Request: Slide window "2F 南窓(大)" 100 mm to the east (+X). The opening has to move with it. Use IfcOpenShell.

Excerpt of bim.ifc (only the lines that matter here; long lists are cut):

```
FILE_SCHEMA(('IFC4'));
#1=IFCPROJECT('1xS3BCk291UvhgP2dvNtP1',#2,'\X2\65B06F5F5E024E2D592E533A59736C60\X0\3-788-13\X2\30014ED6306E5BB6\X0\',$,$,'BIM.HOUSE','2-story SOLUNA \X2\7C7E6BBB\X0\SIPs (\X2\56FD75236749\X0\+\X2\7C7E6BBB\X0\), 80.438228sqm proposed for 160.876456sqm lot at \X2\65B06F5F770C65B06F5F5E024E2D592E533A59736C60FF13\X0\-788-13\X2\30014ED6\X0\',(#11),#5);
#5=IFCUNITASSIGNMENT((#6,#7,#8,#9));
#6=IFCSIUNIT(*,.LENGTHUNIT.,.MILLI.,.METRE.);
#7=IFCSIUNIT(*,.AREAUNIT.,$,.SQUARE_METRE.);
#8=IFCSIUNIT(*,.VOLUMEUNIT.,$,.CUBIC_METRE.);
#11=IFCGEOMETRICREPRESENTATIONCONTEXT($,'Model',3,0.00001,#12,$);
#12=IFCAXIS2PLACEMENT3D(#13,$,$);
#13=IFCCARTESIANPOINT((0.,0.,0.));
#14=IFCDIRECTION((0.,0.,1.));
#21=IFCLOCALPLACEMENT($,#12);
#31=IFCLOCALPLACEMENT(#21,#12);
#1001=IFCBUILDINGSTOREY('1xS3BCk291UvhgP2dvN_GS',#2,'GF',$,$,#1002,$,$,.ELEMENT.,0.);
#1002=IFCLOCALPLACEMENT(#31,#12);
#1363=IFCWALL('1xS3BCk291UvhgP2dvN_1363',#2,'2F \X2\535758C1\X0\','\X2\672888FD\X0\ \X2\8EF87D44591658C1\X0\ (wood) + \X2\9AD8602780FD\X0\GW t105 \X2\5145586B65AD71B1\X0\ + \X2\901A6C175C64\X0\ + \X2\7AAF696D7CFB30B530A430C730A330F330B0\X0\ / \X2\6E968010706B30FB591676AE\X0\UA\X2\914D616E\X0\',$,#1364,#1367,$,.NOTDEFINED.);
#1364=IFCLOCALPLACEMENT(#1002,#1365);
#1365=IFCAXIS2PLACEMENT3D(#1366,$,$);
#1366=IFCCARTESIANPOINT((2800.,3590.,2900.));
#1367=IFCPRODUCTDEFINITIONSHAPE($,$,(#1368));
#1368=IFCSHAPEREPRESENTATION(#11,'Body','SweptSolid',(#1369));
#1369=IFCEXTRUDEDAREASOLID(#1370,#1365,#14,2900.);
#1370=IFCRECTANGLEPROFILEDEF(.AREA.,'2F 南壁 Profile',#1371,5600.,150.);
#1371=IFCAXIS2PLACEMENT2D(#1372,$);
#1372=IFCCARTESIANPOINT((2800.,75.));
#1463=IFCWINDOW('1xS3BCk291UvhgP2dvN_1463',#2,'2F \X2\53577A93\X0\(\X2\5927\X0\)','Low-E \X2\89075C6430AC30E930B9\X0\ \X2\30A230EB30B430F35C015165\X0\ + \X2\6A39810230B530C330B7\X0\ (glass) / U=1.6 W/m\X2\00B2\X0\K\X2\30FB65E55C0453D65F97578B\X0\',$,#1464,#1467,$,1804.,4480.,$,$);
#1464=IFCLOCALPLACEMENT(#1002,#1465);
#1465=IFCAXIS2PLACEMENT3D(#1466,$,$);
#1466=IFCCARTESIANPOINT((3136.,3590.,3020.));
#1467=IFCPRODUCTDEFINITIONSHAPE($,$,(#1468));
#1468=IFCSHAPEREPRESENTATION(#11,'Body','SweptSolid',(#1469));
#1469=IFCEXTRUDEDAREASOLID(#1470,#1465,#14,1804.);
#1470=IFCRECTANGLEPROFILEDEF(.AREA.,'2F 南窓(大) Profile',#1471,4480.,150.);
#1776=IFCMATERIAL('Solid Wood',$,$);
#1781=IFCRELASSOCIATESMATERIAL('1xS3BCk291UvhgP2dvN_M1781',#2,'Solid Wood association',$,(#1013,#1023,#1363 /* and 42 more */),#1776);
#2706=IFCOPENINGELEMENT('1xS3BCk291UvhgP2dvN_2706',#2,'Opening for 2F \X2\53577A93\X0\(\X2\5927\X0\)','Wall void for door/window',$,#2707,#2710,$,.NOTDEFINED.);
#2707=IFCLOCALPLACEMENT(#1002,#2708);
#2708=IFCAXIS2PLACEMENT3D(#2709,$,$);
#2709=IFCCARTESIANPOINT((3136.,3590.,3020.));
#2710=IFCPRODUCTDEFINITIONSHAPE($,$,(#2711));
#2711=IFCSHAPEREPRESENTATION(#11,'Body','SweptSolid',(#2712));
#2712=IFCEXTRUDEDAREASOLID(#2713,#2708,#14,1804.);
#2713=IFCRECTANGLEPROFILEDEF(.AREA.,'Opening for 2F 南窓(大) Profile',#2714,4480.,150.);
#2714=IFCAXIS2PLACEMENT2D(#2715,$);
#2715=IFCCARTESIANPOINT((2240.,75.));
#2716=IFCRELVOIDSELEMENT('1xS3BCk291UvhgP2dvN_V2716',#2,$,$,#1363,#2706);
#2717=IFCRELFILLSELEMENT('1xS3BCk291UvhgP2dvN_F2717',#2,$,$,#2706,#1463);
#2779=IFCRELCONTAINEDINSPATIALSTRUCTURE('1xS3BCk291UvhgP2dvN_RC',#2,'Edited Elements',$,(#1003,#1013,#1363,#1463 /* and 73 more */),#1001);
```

```python
import ifcopenshell
import ifcopenshell.api.geometry
import ifcopenshell.util.placement
import ifcopenshell.util.unit

model = ifcopenshell.open("bim.ifc")
unit_scale = ifcopenshell.util.unit.calculate_unit_scale(model)

window = model.by_id(1463)
opening = window.FillsVoids[0].RelatingOpeningElement
wall = opening.VoidsElements[0].RelatingBuildingElement

wall_matrix = ifcopenshell.util.placement.get_local_placement(wall.ObjectPlacement)
shift = wall_matrix[:3, 0] * 0.1 / unit_scale
before = ifcopenshell.util.placement.get_local_placement(window.ObjectPlacement)[:3, 3].copy()

# The window is not placed relative to its opening, so move both.
for product in (opening, window):
    matrix = ifcopenshell.util.placement.get_local_placement(product.ObjectPlacement)
    matrix[:3, 3] += shift
    ifcopenshell.api.geometry.edit_object_placement(model, product=product, matrix=matrix, is_si=False)

after = ifcopenshell.util.placement.get_local_placement(window.ObjectPlacement)[:3, 3]
print("window moved by", (after - before).round(3) + 0.0)

model.write("bim-out.ifc")
```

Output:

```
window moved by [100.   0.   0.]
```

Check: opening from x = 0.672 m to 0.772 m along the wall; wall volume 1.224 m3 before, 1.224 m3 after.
